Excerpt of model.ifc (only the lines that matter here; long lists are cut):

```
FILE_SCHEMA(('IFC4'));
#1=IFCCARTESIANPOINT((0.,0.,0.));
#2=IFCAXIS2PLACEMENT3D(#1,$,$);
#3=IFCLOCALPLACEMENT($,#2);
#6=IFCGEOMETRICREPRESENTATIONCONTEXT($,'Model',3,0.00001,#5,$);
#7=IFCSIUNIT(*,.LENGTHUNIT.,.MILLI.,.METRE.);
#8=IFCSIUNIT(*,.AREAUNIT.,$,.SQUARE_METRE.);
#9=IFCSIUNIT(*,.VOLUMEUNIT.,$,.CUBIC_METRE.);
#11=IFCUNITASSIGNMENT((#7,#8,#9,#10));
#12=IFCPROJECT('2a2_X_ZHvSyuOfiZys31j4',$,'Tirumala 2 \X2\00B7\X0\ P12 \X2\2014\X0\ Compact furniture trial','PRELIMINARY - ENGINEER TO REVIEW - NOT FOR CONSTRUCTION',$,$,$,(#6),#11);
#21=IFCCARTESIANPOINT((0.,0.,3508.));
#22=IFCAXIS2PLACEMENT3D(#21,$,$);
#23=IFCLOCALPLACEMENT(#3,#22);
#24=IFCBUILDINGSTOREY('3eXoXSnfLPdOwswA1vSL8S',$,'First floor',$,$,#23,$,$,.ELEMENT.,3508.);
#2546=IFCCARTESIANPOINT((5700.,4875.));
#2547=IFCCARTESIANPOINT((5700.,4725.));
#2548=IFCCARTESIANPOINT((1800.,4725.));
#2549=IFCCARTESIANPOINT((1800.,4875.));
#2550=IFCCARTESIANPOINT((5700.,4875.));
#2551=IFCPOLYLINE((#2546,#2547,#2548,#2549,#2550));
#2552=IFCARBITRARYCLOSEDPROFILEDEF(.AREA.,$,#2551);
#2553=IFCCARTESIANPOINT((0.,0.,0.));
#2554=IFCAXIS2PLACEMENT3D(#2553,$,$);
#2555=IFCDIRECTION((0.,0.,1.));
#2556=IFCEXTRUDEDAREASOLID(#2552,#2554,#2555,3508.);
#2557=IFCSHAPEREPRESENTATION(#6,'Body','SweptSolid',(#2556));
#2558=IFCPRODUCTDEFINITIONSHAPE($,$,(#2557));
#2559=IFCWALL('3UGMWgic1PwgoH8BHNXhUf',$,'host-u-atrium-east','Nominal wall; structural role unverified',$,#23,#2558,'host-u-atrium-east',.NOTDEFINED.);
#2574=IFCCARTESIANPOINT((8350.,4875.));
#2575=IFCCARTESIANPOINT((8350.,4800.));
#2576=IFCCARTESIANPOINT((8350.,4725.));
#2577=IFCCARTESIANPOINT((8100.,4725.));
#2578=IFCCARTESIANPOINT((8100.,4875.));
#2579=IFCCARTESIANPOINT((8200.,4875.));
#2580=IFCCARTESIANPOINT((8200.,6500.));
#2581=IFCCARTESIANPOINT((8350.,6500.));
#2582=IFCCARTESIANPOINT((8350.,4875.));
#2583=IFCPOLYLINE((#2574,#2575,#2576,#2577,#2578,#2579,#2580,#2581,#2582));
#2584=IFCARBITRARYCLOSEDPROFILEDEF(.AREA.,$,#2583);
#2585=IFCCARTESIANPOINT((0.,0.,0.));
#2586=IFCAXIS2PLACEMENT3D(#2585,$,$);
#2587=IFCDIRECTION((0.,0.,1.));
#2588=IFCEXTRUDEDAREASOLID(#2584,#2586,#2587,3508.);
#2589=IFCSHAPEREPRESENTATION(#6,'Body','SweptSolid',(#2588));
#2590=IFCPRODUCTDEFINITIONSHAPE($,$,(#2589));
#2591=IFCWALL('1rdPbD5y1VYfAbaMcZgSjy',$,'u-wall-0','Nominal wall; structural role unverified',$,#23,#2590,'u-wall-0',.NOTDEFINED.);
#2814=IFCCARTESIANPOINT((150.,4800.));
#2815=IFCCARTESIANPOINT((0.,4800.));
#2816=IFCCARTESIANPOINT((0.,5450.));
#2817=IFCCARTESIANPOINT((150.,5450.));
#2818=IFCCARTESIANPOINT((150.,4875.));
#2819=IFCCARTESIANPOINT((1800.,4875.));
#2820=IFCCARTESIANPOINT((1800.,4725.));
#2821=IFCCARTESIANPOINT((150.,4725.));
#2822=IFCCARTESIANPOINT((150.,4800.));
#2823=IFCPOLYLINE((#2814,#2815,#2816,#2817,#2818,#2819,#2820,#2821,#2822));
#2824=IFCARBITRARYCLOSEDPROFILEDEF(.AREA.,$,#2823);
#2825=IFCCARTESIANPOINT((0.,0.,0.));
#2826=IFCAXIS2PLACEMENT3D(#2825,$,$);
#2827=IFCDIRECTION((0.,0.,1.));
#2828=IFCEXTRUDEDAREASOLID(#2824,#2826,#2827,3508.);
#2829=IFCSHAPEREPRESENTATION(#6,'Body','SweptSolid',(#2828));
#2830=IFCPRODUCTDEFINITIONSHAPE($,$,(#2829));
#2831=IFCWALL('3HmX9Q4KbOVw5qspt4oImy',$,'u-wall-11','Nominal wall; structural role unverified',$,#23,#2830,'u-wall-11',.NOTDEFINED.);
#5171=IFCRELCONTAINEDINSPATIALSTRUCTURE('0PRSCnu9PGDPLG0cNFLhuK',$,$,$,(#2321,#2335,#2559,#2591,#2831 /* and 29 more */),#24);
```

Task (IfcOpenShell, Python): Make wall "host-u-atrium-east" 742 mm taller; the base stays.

```python
import ifcopenshell
import ifcopenshell.geom
import ifcopenshell.util.shape
import ifcopenshell.util.unit

model = ifcopenshell.open("model.ifc")
unit_scale = ifcopenshell.util.unit.calculate_unit_scale(model)
settings = ifcopenshell.geom.settings()


def volume(element):
    """Net volume in cubic metres, openings subtracted."""
    shape = ifcopenshell.geom.create_shape(settings, element)
    return ifcopenshell.util.shape.get_volume(shape.geometry)


wall = model.by_id(2559)
before = volume(wall)

body = next(r for r in wall.Representation.Representations if r.RepresentationIdentifier == "Body")
solid = body.Items[0]
old_height = solid.Depth
solid.Depth += 0.742 / unit_scale
after = volume(wall)

print(f"height {old_height:g} -> {solid.Depth:g}, volume {before:.3f} -> {after:.3f} m3")

model.write("model_rev.ifc")
```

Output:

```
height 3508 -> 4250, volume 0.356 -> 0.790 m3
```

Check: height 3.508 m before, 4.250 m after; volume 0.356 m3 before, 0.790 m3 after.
